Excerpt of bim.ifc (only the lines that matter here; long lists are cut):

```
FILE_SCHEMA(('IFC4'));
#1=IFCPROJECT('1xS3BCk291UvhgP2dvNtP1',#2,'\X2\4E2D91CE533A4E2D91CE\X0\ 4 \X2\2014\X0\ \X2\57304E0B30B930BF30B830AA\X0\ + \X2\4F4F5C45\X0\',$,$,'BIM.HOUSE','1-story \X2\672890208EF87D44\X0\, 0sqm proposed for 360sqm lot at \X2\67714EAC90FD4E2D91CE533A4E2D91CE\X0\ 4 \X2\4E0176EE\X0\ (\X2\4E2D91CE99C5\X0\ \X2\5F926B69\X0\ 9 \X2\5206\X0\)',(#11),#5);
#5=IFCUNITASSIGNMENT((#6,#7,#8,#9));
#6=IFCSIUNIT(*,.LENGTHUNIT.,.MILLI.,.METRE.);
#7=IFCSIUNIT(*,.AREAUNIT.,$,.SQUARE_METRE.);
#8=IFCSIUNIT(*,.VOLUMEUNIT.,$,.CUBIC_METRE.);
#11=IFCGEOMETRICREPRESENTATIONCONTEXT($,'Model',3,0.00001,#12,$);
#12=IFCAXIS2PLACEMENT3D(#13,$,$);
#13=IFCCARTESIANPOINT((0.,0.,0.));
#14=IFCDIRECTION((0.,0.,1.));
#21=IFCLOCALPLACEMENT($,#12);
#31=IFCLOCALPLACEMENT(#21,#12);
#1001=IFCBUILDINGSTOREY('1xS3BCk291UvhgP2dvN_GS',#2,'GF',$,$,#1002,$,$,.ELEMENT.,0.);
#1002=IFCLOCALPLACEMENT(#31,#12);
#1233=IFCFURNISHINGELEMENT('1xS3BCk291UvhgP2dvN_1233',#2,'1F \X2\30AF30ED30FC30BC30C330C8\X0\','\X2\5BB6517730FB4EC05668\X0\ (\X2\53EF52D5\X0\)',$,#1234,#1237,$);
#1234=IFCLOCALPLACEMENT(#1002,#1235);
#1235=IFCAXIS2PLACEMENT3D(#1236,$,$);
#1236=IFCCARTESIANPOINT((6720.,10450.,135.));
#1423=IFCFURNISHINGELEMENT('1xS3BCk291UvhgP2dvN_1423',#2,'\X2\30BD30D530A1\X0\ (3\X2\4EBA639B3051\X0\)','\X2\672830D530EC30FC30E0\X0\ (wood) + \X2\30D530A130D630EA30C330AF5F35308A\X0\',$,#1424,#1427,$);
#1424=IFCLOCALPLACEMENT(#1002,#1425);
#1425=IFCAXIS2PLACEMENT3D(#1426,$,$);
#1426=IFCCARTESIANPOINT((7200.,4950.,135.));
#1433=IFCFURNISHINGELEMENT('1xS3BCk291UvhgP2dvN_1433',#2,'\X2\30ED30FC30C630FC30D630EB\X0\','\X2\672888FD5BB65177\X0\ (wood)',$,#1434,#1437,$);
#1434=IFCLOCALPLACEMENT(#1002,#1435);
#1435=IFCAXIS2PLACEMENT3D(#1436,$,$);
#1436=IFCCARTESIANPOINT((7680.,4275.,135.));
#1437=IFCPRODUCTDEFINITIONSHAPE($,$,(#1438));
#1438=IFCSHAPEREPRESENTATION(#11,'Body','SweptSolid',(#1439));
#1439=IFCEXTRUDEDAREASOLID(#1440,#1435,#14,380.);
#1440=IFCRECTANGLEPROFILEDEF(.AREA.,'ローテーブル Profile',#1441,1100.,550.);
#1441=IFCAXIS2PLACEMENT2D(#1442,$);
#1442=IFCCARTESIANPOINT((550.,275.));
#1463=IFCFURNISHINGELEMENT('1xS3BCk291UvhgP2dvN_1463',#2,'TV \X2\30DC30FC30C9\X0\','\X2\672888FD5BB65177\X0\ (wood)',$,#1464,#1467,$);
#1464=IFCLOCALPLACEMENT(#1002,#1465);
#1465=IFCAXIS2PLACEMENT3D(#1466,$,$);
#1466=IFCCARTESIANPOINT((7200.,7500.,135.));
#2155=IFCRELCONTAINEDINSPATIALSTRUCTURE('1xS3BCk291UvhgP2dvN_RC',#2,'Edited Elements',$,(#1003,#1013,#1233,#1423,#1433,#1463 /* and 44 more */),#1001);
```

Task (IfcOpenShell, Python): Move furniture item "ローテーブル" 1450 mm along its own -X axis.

```python
import ifcopenshell
import ifcopenshell.api.geometry
import ifcopenshell.util.placement

model = ifcopenshell.open("bim.ifc")

item = model.by_id(1433)
matrix = ifcopenshell.util.placement.get_local_placement(item.ObjectPlacement)
matrix[:3, 3] -= matrix[:3, 0] * 1450.0
ifcopenshell.api.geometry.edit_object_placement(model, product=item, matrix=matrix, is_si=False)

print(ifcopenshell.util.placement.get_local_placement(item.ObjectPlacement).round(3) + 0.0)

model.write("bim_updated.ifc")
```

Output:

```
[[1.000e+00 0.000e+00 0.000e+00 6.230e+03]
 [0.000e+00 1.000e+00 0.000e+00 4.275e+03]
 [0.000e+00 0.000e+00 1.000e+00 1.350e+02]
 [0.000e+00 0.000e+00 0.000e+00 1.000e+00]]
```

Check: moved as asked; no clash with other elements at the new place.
